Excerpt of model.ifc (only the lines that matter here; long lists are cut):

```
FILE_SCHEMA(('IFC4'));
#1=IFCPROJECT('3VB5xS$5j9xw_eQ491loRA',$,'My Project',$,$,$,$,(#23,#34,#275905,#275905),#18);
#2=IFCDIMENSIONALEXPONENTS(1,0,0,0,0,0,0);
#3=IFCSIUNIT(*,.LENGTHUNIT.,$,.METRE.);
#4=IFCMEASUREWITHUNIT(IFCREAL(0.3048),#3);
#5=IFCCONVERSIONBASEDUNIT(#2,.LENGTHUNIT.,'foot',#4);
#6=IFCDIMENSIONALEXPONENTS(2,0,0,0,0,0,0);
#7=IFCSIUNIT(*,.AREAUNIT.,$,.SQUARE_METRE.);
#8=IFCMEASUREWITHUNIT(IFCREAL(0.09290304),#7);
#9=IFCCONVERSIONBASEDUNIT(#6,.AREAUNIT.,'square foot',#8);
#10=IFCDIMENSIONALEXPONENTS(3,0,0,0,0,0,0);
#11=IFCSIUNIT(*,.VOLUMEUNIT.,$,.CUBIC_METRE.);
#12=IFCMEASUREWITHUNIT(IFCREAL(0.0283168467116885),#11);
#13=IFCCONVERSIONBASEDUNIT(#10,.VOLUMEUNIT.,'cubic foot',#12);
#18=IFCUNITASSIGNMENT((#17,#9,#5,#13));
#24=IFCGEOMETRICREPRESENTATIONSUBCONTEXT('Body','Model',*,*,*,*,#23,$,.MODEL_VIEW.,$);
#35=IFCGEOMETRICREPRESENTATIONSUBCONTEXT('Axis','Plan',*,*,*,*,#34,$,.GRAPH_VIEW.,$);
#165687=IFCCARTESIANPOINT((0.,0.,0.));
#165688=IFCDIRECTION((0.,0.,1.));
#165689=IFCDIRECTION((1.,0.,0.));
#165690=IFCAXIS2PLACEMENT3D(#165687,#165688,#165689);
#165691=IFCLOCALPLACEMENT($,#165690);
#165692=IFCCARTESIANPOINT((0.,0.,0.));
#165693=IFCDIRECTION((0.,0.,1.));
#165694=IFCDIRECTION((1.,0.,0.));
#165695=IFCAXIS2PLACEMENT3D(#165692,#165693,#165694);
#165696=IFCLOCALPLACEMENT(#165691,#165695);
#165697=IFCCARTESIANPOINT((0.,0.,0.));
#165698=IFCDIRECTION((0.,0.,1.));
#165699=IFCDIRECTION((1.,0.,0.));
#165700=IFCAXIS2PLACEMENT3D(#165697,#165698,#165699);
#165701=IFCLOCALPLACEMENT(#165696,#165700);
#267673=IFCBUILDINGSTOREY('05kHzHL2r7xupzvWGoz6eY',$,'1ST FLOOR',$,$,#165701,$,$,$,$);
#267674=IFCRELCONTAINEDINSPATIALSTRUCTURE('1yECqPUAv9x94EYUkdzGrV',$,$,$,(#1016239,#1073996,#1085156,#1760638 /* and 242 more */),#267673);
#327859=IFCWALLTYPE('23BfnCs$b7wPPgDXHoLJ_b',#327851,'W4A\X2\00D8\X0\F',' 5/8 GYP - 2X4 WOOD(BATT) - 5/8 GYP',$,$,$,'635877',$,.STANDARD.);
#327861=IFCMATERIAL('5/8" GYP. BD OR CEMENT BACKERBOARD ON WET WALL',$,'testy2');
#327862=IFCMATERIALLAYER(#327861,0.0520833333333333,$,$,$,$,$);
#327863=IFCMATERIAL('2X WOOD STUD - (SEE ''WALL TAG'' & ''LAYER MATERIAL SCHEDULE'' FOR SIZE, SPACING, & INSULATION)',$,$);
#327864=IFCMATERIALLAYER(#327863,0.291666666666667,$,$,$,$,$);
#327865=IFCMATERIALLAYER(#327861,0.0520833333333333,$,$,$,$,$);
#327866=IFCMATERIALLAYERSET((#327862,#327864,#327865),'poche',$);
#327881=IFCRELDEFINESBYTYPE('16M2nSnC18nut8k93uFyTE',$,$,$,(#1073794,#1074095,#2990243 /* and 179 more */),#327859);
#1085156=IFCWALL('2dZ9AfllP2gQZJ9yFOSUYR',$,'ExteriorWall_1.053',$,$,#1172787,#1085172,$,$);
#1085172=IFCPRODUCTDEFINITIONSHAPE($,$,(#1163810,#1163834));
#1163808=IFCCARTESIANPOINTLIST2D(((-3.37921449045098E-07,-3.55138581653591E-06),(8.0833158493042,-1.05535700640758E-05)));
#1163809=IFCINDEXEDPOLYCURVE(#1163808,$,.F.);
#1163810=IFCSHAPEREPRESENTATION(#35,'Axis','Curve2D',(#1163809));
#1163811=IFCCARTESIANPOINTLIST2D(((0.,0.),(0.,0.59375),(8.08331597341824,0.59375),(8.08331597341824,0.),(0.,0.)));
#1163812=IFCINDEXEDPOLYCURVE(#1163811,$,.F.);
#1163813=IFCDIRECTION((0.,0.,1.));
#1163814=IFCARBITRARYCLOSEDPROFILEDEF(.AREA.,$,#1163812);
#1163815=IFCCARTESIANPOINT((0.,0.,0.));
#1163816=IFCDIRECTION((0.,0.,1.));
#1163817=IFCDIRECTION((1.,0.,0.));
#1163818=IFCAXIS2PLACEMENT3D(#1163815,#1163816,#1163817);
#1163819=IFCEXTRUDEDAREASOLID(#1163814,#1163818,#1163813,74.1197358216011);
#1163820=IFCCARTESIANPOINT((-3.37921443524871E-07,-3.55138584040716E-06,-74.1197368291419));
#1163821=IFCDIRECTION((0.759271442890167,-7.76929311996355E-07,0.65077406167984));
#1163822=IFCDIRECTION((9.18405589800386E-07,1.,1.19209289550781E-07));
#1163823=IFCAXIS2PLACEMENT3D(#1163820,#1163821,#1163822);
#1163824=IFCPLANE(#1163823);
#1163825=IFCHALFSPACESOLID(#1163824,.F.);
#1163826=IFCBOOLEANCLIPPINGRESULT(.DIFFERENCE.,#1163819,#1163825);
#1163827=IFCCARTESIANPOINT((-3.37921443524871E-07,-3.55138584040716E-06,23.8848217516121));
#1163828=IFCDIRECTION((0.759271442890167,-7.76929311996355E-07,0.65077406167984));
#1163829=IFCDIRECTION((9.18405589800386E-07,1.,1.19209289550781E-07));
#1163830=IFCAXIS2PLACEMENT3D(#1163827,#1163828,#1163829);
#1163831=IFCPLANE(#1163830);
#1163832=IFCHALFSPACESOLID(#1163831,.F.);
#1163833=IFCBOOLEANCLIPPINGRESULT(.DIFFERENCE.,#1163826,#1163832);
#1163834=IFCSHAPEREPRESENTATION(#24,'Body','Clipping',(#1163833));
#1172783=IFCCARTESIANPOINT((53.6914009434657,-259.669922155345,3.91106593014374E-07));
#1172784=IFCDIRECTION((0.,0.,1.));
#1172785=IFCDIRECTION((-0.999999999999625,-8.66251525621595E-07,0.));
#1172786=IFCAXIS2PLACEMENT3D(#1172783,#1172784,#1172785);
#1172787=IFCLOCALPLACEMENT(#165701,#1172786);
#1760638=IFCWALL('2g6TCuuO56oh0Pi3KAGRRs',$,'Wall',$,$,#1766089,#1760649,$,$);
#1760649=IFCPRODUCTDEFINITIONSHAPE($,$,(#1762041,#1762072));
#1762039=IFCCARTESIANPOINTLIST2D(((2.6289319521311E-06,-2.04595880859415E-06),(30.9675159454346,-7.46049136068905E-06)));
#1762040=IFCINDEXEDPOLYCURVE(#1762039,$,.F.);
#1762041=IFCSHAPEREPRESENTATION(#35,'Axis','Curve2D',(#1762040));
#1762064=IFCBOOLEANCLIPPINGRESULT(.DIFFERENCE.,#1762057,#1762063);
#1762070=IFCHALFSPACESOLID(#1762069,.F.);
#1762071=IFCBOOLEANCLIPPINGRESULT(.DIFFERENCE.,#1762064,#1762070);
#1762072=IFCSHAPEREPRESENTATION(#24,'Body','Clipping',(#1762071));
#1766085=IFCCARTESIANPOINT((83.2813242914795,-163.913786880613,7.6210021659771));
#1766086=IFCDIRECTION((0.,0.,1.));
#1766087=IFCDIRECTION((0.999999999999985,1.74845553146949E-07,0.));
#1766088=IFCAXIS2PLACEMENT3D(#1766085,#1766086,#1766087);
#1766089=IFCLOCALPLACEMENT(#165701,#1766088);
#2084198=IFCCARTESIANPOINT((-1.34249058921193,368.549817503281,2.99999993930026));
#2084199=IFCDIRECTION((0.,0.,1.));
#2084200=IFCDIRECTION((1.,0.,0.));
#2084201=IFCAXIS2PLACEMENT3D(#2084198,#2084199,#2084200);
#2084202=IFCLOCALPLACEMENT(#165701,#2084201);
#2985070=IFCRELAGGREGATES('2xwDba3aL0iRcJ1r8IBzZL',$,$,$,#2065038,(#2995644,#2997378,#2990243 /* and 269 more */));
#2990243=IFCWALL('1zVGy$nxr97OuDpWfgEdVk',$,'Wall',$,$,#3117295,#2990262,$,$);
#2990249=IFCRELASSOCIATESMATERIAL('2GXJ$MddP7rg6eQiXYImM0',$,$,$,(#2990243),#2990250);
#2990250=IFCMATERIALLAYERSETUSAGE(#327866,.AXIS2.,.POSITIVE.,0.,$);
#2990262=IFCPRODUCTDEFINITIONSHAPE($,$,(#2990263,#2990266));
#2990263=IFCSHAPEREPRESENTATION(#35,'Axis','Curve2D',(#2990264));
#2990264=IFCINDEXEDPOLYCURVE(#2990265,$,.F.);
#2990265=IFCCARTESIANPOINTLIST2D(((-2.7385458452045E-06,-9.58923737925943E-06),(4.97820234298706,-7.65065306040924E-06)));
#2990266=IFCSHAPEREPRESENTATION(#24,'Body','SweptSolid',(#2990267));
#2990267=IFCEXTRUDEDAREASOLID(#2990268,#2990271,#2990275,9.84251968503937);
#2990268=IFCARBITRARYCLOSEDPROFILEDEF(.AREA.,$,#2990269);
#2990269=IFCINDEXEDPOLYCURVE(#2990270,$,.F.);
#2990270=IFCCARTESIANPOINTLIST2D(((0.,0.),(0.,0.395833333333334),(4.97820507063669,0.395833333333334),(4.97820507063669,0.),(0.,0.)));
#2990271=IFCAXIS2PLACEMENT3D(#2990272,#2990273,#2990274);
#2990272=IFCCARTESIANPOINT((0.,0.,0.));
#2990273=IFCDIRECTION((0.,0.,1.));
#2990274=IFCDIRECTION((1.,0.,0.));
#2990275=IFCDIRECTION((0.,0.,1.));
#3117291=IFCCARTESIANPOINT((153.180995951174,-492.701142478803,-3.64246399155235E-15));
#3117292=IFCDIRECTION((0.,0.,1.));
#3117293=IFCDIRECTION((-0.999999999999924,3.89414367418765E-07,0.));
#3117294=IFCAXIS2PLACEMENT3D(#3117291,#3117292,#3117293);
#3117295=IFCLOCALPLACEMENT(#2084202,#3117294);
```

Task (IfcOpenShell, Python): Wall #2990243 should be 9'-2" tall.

```python
import ifcopenshell
import ifcopenshell.geom
import ifcopenshell.util.representation
import ifcopenshell.util.shape
import ifcopenshell.util.unit

model = ifcopenshell.open("model.ifc")
unit_scale = ifcopenshell.util.unit.calculate_unit_scale(model)
settings = ifcopenshell.geom.settings()


def volume(element):
    """Net volume in cubic metres, openings subtracted."""
    shape = ifcopenshell.geom.create_shape(settings, element)
    return ifcopenshell.util.shape.get_volume(shape.geometry)


wall = model.by_guid("1zVGy$nxr97OuDpWfgEdVk")
before = volume(wall)

body = ifcopenshell.util.representation.get_representation(wall, "Model", "Body")
solid = body.Items[0]
old_height = solid.Depth
solid.Depth = 110 * 0.0254 / unit_scale
after = volume(wall)

print(f"height {old_height:g} -> {solid.Depth:g}, volume {before:.3f} -> {after:.3f} m3")

model.write("model_rev.ifc")
```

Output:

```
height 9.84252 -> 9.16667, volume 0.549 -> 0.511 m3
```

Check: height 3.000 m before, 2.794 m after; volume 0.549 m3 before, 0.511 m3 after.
